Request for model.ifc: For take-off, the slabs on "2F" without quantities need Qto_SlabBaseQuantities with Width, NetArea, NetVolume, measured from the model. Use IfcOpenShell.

First a look at what the model holds.

```python
import ifcopenshell
import ifcopenshell.util.element
import ifcopenshell.util.unit

model = ifcopenshell.open("model.ifc")
print(model.schema)
for unit_type in ("LENGTHUNIT", "AREAUNIT", "VOLUMEUNIT"):
    print(unit_type, ifcopenshell.util.unit.calculate_unit_scale(model, unit_type))
storey = next(s for s in model.by_type("IfcBuildingStorey") if s.Name == "2F")
slabs = [e for e in ifcopenshell.util.element.get_decomposition(storey) if e.is_a("IfcSlab")]
for e in sorted(slabs, key=lambda e: e.id()):
    print(e.id(), e.is_a(), e.Name, list(ifcopenshell.util.element.get_psets(e, qtos_only=True)), sep=" | ")
```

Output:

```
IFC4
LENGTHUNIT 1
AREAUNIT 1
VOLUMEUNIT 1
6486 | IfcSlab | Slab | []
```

```python
import ifcopenshell
import ifcopenshell.api.pset
import ifcopenshell.geom
import ifcopenshell.util.element
import ifcopenshell.util.shape
import ifcopenshell.util.unit

model = ifcopenshell.open("model.ifc")
unit_scale = ifcopenshell.util.unit.calculate_unit_scale(model)
area_scale = ifcopenshell.util.unit.calculate_unit_scale(model, "AREAUNIT")
volume_scale = ifcopenshell.util.unit.calculate_unit_scale(model, "VOLUMEUNIT")
settings = ifcopenshell.geom.settings()

storey = next(s for s in model.by_type("IfcBuildingStorey") if s.Name == "2F")
slabs = [e for e in ifcopenshell.util.element.get_decomposition(storey) if e.is_a("IfcSlab")]

for e in sorted(slabs, key=lambda e: e.id()):
    if ifcopenshell.util.element.get_psets(e, qtos_only=True, should_inherit=False):
        continue
    # Geometry comes back in metres, in the element's own axes.
    shape = ifcopenshell.geom.create_shape(settings, e)
    values = {
        "Width": ifcopenshell.util.shape.get_z(shape.geometry) / unit_scale,
        "NetArea": ifcopenshell.util.shape.get_footprint_area(shape.geometry) / area_scale,
        "NetVolume": ifcopenshell.util.shape.get_volume(shape.geometry) / volume_scale,
    }
    qto = ifcopenshell.api.pset.add_qto(model, product=e, name="Qto_SlabBaseQuantities")
    ifcopenshell.api.pset.edit_qto(model, qto=qto, properties=values)
    print(e.id(), {k: round(v, 3) for k, v in values.items()})

model.write("model_v2.ifc")
```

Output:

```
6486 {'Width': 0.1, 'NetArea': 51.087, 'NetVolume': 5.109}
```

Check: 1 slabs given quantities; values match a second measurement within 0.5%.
